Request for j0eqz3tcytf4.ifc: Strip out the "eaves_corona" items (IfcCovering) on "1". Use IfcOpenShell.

First a look at what the model holds.

```python
import ifcopenshell
import ifcopenshell.util.element

model = ifcopenshell.open("j0eqz3tcytf4.ifc")
print(model.schema)
storey = next(s for s in model.by_type("IfcBuildingStorey") if s.Name == "1")
coverings = [e for e in ifcopenshell.util.element.get_decomposition(storey) if e.is_a("IfcCovering")]
seen = {}
for e in coverings:
    element_type = ifcopenshell.util.element.get_type(e)
    name = element_type.Name if element_type not in (None, e) else None
    seen[name] = seen.get(name, 0) + 1
for name, count in sorted(seen.items(), key=str):
    print(count, "x", name)
```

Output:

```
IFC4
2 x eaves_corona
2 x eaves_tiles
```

```python
import ifcopenshell
import ifcopenshell.api.root
import ifcopenshell.util.element

model = ifcopenshell.open("j0eqz3tcytf4.ifc")

storey = next(s for s in model.by_type("IfcBuildingStorey") if s.Name == "1")
coverings = [e for e in ifcopenshell.util.element.get_decomposition(storey) if e.is_a("IfcCovering")]
targets = [e for e in coverings if (t := ifcopenshell.util.element.get_type(e)) not in (None, e) and t.Name == "eaves_corona"]

for e in targets:
    ifcopenshell.api.root.remove_product(model, product=e)
print(len(targets), "removed")

model.write("j0eqz3tcytf4_rev.ifc")
```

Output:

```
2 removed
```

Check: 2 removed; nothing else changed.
